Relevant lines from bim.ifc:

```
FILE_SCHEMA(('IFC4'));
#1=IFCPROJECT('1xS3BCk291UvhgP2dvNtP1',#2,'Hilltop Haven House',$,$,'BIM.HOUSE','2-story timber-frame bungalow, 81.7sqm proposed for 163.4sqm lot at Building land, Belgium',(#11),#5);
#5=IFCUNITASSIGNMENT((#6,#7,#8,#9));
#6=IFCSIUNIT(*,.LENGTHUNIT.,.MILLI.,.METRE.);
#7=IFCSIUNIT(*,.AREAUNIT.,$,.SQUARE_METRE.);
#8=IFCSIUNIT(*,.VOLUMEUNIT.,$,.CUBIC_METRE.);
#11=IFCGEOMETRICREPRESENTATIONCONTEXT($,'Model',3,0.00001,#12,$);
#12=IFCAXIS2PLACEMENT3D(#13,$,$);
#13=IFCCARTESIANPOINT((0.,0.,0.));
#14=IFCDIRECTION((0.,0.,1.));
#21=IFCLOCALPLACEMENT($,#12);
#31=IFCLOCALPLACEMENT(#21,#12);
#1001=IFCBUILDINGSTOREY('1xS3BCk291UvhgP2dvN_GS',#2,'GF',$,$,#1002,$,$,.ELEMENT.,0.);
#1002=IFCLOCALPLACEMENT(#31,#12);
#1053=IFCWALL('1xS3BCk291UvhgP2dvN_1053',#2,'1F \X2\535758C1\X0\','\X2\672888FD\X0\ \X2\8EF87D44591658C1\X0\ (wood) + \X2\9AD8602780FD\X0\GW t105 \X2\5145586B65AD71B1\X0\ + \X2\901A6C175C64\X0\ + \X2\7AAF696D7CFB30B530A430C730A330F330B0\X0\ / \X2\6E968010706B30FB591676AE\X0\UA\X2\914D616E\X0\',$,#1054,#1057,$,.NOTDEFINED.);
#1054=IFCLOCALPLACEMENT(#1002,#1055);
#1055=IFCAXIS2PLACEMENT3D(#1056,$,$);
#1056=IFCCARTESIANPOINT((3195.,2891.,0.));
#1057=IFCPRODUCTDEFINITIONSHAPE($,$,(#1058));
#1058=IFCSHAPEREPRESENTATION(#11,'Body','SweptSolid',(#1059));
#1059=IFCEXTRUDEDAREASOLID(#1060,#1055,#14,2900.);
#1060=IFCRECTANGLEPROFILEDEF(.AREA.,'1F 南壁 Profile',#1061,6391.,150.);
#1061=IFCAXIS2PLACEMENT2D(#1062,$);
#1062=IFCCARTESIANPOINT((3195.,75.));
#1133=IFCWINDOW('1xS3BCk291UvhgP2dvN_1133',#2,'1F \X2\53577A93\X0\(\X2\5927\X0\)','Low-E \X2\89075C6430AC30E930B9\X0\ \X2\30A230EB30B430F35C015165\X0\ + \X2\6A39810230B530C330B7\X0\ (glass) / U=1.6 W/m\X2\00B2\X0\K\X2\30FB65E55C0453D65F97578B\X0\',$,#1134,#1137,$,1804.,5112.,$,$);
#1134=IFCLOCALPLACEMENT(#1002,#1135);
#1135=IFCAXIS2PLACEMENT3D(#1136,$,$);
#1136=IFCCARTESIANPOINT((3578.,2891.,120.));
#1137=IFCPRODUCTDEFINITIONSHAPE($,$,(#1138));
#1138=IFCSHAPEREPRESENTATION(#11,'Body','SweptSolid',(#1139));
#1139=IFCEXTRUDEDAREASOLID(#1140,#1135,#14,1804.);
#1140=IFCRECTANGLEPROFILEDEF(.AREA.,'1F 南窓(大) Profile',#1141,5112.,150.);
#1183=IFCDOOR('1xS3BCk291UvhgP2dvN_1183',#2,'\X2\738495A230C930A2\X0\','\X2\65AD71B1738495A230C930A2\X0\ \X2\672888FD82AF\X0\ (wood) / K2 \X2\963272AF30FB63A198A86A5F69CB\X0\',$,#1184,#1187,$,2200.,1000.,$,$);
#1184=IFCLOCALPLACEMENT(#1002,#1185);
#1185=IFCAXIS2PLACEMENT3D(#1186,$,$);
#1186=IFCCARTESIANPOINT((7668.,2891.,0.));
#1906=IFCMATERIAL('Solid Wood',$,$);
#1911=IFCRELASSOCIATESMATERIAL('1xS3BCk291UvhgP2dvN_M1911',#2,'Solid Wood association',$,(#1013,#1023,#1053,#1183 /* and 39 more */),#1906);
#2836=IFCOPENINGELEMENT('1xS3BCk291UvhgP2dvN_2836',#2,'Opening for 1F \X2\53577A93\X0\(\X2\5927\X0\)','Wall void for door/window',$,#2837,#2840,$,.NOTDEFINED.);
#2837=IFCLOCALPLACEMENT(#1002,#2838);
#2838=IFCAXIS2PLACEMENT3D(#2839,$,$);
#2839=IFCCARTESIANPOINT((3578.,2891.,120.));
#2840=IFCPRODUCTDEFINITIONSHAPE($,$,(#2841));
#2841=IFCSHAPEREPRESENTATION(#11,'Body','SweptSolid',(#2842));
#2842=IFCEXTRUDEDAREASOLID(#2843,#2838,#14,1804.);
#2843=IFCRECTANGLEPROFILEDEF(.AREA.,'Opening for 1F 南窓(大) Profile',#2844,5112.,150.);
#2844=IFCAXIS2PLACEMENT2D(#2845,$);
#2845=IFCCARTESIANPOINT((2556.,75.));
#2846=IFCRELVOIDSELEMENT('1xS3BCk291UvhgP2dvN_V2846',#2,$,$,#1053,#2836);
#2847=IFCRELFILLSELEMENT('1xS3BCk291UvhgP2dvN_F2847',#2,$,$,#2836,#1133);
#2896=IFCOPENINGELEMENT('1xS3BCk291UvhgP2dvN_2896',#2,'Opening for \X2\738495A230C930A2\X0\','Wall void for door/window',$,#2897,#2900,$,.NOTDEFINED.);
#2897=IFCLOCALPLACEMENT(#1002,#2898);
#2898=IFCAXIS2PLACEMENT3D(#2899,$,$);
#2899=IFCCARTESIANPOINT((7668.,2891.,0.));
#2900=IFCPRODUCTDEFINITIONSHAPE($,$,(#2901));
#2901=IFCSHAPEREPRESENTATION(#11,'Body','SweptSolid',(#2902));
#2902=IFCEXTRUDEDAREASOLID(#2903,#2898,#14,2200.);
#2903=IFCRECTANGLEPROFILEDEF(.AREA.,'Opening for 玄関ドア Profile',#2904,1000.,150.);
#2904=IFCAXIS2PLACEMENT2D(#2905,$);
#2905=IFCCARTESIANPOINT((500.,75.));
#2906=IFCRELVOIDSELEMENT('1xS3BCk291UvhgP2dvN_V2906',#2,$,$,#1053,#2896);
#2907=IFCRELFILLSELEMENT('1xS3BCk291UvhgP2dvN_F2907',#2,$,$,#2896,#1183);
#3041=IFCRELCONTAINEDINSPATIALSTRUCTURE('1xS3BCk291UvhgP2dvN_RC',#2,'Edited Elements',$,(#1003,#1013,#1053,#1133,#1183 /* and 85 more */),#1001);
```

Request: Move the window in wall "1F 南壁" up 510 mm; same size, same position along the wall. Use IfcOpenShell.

```python
import numpy as np
import ifcopenshell
import ifcopenshell.api.geometry
import ifcopenshell.util.placement
import ifcopenshell.util.unit

model = ifcopenshell.open("bim.ifc")
unit_scale = ifcopenshell.util.unit.calculate_unit_scale(model)

window = model.by_id(1133)
opening = window.FillsVoids[0].RelatingOpeningElement
dz = 510.0

shift = np.array([0.0, 0.0, dz])
# The window is not placed relative to its opening, so move both.
for product in (opening, window):
    matrix = ifcopenshell.util.placement.get_local_placement(product.ObjectPlacement)
    matrix[:3, 3] += shift
    ifcopenshell.api.geometry.edit_object_placement(model, product=product, matrix=matrix, is_si=False)

print(f"moved by {dz * unit_scale:+.3f} m")

model.write("bim_v2.ifc")
```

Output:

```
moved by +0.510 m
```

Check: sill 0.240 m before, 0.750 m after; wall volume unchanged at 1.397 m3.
